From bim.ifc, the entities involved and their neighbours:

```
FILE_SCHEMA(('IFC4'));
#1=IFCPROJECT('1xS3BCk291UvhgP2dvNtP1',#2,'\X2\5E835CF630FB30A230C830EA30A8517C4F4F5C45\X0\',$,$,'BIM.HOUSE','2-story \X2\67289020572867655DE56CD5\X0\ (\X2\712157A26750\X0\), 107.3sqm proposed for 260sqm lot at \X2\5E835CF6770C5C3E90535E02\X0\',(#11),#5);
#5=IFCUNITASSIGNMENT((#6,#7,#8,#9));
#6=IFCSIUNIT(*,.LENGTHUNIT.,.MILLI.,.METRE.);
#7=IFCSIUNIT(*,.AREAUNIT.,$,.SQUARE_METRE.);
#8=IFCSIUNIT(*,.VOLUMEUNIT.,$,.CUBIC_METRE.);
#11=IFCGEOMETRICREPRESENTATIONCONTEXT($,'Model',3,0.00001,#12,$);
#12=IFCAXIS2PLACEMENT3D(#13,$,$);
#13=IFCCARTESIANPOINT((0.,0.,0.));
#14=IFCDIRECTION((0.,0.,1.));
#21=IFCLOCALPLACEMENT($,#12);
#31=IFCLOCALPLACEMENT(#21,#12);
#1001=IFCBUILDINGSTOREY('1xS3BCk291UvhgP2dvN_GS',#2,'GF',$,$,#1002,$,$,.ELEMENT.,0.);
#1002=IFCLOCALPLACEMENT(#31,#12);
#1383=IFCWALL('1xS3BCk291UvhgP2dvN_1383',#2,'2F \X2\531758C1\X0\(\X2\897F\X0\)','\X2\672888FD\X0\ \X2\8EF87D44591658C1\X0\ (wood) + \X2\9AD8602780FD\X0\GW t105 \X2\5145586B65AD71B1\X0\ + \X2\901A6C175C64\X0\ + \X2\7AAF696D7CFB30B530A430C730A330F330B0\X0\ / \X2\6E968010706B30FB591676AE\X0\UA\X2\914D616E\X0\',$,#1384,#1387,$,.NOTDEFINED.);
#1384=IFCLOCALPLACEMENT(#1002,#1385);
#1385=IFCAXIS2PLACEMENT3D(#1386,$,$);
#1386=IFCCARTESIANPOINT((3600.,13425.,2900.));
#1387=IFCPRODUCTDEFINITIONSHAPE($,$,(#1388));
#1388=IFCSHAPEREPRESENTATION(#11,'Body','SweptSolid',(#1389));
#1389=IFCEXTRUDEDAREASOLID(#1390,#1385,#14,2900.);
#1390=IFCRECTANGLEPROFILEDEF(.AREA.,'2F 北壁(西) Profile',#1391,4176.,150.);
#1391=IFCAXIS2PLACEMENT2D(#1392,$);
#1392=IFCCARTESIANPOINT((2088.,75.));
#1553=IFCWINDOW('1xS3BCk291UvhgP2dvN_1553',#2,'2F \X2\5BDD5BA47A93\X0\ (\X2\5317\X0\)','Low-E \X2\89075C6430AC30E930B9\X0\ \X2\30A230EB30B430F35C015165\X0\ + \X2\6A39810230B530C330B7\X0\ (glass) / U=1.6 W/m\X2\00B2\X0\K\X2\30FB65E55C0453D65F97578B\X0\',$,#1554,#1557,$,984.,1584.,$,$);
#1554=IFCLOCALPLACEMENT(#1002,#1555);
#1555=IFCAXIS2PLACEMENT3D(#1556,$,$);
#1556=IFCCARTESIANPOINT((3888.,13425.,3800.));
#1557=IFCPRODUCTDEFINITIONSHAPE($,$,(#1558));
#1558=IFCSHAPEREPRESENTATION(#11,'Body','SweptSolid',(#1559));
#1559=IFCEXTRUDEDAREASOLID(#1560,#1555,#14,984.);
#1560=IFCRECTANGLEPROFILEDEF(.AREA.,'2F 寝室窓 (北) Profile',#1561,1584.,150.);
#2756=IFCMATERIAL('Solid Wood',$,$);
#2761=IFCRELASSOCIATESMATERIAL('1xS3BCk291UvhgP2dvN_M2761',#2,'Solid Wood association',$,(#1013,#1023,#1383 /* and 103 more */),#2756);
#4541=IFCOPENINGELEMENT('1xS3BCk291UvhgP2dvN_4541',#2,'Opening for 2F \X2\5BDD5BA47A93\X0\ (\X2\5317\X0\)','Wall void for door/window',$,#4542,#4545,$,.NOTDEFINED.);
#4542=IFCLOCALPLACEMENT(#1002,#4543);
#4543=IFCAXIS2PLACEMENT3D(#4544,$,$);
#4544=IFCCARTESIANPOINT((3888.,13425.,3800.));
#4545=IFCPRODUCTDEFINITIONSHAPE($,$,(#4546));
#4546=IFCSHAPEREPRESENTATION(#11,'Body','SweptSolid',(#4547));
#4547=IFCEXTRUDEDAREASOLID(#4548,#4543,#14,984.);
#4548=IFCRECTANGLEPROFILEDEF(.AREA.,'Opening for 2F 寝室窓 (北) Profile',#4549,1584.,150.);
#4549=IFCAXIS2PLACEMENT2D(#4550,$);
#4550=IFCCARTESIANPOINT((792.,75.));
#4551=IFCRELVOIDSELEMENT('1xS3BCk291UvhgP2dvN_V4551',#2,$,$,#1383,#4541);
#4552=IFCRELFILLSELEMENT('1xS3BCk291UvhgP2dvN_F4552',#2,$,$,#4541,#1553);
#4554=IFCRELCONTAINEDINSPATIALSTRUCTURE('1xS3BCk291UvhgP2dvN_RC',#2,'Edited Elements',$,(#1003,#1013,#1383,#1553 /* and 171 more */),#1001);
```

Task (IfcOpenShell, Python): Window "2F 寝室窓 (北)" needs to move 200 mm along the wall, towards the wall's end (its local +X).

```python
import ifcopenshell
import ifcopenshell.api.geometry
import ifcopenshell.util.placement

model = ifcopenshell.open("bim.ifc")

window = model.by_id(1553)
opening = window.FillsVoids[0].RelatingOpeningElement
wall = opening.VoidsElements[0].RelatingBuildingElement

wall_matrix = ifcopenshell.util.placement.get_local_placement(wall.ObjectPlacement)
shift = wall_matrix[:3, 0] * 200.0
before = ifcopenshell.util.placement.get_local_placement(window.ObjectPlacement)[:3, 3].copy()

# The window is not placed relative to its opening, so move both.
for product in (opening, window):
    matrix = ifcopenshell.util.placement.get_local_placement(product.ObjectPlacement)
    matrix[:3, 3] += shift
    ifcopenshell.api.geometry.edit_object_placement(model, product=product, matrix=matrix, is_si=False)

after = ifcopenshell.util.placement.get_local_placement(window.ObjectPlacement)[:3, 3]
print("window moved by", (after - before).round(3) + 0.0)

model.write("bim_updated.ifc")
```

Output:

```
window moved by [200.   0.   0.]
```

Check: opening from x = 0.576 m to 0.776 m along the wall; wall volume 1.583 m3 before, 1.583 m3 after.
